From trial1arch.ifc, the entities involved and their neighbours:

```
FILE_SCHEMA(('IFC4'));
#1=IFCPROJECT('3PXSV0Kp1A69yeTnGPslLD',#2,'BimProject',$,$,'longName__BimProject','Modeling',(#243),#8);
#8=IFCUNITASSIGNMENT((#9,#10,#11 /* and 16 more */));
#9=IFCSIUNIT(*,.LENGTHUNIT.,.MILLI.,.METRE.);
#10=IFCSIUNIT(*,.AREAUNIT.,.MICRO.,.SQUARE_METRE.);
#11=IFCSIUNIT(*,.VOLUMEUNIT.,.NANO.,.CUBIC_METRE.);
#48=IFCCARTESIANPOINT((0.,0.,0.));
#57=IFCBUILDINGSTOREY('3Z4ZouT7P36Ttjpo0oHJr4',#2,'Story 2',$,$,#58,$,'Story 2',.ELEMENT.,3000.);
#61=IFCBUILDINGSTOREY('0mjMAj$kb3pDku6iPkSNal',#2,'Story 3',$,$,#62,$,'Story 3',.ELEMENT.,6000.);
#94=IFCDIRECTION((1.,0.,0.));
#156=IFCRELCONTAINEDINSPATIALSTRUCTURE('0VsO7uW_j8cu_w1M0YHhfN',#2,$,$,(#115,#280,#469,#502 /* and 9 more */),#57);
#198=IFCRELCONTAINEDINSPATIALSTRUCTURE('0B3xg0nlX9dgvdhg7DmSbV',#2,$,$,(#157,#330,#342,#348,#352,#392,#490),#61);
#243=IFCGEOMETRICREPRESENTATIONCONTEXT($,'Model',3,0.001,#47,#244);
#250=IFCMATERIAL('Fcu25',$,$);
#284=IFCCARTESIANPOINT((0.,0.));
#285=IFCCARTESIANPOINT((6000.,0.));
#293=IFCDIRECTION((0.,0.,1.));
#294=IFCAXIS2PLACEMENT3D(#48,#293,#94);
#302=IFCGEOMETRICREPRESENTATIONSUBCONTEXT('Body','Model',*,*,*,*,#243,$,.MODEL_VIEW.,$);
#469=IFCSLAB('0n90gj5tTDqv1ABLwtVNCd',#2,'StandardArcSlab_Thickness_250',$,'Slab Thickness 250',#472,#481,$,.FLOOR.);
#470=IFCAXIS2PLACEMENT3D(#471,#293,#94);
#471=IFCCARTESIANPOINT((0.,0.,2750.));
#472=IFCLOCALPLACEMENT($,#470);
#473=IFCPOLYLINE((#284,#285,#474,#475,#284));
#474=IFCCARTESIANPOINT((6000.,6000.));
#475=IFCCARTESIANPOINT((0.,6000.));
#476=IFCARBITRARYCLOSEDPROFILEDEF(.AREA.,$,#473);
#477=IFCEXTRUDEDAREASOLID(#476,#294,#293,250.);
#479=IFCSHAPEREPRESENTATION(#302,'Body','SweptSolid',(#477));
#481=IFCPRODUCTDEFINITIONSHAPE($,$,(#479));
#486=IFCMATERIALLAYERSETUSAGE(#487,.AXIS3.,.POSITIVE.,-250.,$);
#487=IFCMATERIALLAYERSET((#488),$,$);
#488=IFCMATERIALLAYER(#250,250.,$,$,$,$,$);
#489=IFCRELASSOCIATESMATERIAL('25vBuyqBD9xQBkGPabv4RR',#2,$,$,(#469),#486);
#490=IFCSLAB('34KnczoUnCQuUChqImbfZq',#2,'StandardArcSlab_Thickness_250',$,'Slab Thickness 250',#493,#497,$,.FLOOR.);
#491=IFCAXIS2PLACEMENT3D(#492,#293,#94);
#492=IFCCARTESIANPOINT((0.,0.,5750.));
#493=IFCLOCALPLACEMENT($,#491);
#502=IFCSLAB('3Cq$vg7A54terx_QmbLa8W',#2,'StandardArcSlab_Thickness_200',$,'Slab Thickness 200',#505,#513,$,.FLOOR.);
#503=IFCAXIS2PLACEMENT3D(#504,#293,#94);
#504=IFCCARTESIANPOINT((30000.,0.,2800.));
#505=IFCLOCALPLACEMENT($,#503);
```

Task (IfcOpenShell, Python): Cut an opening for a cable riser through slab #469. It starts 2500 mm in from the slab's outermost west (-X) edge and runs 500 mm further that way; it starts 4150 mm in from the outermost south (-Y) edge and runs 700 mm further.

```python
import numpy as np
import ifcopenshell
import ifcopenshell.api.feature
import ifcopenshell.api.geometry
import ifcopenshell.api.root
import ifcopenshell.geom
import ifcopenshell.util.placement
import ifcopenshell.util.representation
import ifcopenshell.util.shape
import ifcopenshell.util.unit

model = ifcopenshell.open("trial1arch.ifc")
unit_scale = ifcopenshell.util.unit.calculate_unit_scale(model)
settings = ifcopenshell.geom.settings()


def volume(element):
    """Net volume in cubic metres, openings subtracted."""
    shape = ifcopenshell.geom.create_shape(settings, element)
    return ifcopenshell.util.shape.get_volume(shape.geometry)


slab = model.by_guid("0n90gj5tTDqv1ABLwtVNCd")
before = volume(slab)

# Extent in the slab's own axes, in metres. The edges named are its -X and -Y sides.
slab_shape = ifcopenshell.geom.create_shape(settings, slab)
vertices = ifcopenshell.util.shape.get_vertices(slab_shape.geometry)
x_min, y_min, bottom = vertices.min(axis=0)
top = vertices[:, 2].max()

opening = ifcopenshell.api.root.create_entity(model, ifc_class="IfcOpeningElement", name="Cable riser opening", predefined_type="OPENING")
context = ifcopenshell.util.representation.get_context(model, "Model", "Body", "MODEL_VIEW")
width, depth = 0.5, 0.7
outline = [(0.0, 0.0), (width, 0.0), (width, depth), (0.0, depth), (0.0, 0.0)]
# Overshoot both faces by 50 mm so the cut is clean.
shape = ifcopenshell.api.geometry.add_slab_representation(
    model, context=context, depth=top - bottom + 0.1, polyline=outline
)
ifcopenshell.api.geometry.assign_representation(model, product=opening, representation=shape)

matrix = ifcopenshell.util.placement.get_local_placement(slab.ObjectPlacement)
matrix[:, 3] = matrix @ np.append(np.array([x_min + 2.5, y_min + 4.15, bottom - 0.05]) / unit_scale, 1.0)
ifcopenshell.api.geometry.edit_object_placement(model, product=opening, matrix=matrix, is_si=False)
ifcopenshell.api.feature.add_feature(model, feature=opening, element=slab)

after = volume(slab)

print(f"slab volume {before:.3f} -> {after:.3f} m3")

model.write("trial1arch_updated.ifc")
```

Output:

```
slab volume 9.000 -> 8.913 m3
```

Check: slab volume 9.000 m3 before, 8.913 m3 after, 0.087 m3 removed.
